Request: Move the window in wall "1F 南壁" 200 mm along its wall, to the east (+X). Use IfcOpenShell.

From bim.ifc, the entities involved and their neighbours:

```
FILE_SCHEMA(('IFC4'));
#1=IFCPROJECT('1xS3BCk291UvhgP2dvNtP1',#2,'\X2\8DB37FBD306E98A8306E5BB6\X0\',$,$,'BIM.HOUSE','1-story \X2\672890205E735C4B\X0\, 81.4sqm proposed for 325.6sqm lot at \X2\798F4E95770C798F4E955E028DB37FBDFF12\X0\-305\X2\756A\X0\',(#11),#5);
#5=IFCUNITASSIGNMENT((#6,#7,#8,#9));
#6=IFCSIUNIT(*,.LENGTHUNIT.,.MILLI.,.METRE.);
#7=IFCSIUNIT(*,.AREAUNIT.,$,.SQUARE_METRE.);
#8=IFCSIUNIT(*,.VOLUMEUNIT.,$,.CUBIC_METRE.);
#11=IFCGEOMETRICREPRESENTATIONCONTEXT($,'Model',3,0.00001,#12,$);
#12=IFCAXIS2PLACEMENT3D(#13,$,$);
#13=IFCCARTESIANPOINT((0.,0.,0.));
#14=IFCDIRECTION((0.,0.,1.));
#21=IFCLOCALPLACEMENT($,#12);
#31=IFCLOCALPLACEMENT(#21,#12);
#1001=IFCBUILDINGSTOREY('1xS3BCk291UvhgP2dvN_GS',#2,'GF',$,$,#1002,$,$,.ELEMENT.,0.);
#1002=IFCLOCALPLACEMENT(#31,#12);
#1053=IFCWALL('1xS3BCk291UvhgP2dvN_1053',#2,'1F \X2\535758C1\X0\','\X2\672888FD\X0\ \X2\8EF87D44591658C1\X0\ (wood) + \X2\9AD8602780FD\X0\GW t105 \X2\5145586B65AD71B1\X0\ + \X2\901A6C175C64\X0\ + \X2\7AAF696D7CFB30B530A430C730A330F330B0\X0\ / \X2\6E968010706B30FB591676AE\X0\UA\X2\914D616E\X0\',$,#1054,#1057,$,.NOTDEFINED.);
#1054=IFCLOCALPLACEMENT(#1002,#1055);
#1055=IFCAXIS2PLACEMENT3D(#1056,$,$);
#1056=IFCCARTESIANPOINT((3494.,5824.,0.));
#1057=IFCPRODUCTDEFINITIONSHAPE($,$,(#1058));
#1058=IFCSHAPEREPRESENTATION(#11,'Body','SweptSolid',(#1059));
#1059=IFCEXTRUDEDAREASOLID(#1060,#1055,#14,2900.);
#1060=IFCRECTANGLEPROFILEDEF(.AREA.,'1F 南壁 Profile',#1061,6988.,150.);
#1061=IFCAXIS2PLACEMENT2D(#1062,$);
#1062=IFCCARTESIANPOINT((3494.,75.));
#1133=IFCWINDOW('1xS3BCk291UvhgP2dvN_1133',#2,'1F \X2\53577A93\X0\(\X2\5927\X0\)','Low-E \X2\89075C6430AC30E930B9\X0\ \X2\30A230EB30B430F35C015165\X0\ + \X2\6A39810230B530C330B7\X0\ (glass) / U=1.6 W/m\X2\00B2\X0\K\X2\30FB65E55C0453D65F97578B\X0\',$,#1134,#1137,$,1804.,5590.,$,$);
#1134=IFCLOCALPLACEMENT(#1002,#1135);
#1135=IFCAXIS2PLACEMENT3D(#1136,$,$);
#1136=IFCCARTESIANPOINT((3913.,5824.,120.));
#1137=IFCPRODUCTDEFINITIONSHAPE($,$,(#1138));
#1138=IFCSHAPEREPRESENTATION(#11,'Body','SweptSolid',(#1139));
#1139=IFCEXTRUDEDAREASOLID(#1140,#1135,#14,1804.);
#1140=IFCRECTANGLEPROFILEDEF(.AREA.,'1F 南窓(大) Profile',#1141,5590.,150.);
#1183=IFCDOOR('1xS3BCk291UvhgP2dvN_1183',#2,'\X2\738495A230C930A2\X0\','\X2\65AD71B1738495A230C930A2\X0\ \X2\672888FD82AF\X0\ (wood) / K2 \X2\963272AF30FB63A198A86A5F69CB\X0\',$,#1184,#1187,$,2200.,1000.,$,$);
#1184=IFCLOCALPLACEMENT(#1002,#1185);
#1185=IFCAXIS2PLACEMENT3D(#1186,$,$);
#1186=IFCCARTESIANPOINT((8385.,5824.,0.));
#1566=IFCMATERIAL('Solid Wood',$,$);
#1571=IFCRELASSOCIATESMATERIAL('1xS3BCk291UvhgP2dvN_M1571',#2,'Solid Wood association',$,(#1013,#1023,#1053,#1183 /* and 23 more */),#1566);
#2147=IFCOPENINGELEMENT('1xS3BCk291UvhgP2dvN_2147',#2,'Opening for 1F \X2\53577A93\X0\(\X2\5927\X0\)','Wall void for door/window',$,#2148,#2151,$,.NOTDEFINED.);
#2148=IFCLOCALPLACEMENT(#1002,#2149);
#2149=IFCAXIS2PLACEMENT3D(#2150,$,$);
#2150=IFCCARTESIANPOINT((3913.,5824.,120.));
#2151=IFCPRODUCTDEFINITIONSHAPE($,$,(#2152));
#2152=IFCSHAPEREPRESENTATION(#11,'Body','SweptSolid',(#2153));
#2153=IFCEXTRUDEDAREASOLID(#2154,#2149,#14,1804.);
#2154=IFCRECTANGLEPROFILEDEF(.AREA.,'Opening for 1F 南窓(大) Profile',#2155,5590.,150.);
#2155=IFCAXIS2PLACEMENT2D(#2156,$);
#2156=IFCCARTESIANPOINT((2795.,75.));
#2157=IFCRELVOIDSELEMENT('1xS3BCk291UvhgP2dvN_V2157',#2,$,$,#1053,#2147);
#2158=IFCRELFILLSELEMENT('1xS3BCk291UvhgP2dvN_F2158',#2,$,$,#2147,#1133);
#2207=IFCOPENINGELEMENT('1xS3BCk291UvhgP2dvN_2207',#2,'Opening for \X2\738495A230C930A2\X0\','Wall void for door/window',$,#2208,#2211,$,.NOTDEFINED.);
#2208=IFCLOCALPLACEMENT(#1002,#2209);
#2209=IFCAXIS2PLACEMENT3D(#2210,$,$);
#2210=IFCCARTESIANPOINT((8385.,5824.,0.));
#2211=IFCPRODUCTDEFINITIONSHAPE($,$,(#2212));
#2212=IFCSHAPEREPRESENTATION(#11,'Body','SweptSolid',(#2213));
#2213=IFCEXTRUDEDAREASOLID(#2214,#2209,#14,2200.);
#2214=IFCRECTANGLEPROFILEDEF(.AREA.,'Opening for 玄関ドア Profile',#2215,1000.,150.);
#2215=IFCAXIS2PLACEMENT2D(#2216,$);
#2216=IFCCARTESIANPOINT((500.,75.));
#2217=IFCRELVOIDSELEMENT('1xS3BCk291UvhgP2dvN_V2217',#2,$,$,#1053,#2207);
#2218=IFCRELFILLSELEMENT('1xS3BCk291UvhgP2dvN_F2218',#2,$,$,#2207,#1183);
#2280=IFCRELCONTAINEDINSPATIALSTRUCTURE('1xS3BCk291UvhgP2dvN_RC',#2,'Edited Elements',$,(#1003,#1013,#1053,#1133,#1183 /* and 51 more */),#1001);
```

```python
import ifcopenshell
import ifcopenshell.api.geometry
import ifcopenshell.util.placement
import ifcopenshell.util.unit

model = ifcopenshell.open("bim.ifc")
unit_scale = ifcopenshell.util.unit.calculate_unit_scale(model)

window = model.by_guid("1xS3BCk291UvhgP2dvN_1133")
opening = window.FillsVoids[0].RelatingOpeningElement
wall = opening.VoidsElements[0].RelatingBuildingElement

wall_matrix = ifcopenshell.util.placement.get_local_placement(wall.ObjectPlacement)
shift = wall_matrix[:3, 0] * 0.2 / unit_scale
before = ifcopenshell.util.placement.get_local_placement(window.ObjectPlacement)[:3, 3].copy()

# The window is not placed relative to its opening, so move both.
for product in (opening, window):
    matrix = ifcopenshell.util.placement.get_local_placement(product.ObjectPlacement)
    matrix[:3, 3] += shift
    ifcopenshell.api.geometry.edit_object_placement(model, product=product, matrix=matrix, is_si=False)

after = ifcopenshell.util.placement.get_local_placement(window.ObjectPlacement)[:3, 3]
print("window moved by", (after - before).round(3) + 0.0)

model.write("bim_updated.ifc")
```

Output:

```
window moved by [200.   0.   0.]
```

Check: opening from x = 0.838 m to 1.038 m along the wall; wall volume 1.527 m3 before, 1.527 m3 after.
